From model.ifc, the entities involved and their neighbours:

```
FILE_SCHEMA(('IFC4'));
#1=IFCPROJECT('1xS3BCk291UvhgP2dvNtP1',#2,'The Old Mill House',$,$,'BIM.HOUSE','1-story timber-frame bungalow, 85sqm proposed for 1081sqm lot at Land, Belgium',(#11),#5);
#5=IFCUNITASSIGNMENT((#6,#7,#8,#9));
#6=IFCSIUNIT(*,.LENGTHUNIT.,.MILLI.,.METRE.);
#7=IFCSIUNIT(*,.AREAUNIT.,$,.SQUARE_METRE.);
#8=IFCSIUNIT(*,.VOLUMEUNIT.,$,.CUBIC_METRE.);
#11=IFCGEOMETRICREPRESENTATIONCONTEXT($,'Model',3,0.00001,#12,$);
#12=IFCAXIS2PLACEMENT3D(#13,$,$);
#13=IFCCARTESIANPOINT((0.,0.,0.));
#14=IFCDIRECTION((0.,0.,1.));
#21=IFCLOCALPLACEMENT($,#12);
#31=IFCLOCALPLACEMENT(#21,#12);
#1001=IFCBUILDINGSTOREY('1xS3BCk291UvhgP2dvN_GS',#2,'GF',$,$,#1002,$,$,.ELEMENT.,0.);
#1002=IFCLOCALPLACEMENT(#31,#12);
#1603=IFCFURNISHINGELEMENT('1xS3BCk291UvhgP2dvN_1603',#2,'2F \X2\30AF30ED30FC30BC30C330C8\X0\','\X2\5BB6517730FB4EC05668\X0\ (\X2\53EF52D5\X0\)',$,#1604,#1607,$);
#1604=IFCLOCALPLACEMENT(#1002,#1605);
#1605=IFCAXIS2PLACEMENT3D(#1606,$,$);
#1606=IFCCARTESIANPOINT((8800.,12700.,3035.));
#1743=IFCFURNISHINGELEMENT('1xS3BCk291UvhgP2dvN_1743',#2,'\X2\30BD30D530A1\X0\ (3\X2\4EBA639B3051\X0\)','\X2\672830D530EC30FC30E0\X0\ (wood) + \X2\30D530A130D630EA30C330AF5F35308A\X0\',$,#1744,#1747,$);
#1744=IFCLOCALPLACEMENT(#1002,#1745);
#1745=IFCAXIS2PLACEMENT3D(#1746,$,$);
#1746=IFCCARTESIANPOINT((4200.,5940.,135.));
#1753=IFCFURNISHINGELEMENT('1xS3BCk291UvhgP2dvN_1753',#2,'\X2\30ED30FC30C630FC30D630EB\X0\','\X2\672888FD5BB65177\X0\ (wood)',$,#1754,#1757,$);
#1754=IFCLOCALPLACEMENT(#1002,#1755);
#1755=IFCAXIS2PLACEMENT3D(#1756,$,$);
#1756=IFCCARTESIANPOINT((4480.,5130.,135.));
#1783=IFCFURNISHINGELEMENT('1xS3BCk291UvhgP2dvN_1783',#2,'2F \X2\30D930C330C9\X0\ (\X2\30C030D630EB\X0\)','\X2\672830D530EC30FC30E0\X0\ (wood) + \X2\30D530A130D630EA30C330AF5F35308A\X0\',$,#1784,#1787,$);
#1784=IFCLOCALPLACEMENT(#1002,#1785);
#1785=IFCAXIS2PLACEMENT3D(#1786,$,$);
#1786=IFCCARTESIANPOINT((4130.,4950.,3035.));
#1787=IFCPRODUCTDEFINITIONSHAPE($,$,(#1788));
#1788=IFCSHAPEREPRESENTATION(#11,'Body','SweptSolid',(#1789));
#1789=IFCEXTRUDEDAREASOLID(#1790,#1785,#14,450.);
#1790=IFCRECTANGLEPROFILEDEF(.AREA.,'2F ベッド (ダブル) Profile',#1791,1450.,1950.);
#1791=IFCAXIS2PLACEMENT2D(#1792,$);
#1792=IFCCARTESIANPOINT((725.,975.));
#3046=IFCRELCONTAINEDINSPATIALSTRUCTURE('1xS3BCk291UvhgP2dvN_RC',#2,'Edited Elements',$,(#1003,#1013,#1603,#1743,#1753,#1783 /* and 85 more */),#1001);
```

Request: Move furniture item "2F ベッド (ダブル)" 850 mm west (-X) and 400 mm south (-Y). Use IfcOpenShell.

```python
import ifcopenshell
import ifcopenshell.api.geometry
import ifcopenshell.util.placement

model = ifcopenshell.open("model.ifc")

item = model.by_guid("1xS3BCk291UvhgP2dvN_1783")
matrix = ifcopenshell.util.placement.get_local_placement(item.ObjectPlacement)
matrix[0, 3] -= 850.0
matrix[1, 3] -= 400.0
ifcopenshell.api.geometry.edit_object_placement(model, product=item, matrix=matrix, is_si=False)

print(ifcopenshell.util.placement.get_local_placement(item.ObjectPlacement).round(3) + 0.0)

model.write("model-out.ifc")
```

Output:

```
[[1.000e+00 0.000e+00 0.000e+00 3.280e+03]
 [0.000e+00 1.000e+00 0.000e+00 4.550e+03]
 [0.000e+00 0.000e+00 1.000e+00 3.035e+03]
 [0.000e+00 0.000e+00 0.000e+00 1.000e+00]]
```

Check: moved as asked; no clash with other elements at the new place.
